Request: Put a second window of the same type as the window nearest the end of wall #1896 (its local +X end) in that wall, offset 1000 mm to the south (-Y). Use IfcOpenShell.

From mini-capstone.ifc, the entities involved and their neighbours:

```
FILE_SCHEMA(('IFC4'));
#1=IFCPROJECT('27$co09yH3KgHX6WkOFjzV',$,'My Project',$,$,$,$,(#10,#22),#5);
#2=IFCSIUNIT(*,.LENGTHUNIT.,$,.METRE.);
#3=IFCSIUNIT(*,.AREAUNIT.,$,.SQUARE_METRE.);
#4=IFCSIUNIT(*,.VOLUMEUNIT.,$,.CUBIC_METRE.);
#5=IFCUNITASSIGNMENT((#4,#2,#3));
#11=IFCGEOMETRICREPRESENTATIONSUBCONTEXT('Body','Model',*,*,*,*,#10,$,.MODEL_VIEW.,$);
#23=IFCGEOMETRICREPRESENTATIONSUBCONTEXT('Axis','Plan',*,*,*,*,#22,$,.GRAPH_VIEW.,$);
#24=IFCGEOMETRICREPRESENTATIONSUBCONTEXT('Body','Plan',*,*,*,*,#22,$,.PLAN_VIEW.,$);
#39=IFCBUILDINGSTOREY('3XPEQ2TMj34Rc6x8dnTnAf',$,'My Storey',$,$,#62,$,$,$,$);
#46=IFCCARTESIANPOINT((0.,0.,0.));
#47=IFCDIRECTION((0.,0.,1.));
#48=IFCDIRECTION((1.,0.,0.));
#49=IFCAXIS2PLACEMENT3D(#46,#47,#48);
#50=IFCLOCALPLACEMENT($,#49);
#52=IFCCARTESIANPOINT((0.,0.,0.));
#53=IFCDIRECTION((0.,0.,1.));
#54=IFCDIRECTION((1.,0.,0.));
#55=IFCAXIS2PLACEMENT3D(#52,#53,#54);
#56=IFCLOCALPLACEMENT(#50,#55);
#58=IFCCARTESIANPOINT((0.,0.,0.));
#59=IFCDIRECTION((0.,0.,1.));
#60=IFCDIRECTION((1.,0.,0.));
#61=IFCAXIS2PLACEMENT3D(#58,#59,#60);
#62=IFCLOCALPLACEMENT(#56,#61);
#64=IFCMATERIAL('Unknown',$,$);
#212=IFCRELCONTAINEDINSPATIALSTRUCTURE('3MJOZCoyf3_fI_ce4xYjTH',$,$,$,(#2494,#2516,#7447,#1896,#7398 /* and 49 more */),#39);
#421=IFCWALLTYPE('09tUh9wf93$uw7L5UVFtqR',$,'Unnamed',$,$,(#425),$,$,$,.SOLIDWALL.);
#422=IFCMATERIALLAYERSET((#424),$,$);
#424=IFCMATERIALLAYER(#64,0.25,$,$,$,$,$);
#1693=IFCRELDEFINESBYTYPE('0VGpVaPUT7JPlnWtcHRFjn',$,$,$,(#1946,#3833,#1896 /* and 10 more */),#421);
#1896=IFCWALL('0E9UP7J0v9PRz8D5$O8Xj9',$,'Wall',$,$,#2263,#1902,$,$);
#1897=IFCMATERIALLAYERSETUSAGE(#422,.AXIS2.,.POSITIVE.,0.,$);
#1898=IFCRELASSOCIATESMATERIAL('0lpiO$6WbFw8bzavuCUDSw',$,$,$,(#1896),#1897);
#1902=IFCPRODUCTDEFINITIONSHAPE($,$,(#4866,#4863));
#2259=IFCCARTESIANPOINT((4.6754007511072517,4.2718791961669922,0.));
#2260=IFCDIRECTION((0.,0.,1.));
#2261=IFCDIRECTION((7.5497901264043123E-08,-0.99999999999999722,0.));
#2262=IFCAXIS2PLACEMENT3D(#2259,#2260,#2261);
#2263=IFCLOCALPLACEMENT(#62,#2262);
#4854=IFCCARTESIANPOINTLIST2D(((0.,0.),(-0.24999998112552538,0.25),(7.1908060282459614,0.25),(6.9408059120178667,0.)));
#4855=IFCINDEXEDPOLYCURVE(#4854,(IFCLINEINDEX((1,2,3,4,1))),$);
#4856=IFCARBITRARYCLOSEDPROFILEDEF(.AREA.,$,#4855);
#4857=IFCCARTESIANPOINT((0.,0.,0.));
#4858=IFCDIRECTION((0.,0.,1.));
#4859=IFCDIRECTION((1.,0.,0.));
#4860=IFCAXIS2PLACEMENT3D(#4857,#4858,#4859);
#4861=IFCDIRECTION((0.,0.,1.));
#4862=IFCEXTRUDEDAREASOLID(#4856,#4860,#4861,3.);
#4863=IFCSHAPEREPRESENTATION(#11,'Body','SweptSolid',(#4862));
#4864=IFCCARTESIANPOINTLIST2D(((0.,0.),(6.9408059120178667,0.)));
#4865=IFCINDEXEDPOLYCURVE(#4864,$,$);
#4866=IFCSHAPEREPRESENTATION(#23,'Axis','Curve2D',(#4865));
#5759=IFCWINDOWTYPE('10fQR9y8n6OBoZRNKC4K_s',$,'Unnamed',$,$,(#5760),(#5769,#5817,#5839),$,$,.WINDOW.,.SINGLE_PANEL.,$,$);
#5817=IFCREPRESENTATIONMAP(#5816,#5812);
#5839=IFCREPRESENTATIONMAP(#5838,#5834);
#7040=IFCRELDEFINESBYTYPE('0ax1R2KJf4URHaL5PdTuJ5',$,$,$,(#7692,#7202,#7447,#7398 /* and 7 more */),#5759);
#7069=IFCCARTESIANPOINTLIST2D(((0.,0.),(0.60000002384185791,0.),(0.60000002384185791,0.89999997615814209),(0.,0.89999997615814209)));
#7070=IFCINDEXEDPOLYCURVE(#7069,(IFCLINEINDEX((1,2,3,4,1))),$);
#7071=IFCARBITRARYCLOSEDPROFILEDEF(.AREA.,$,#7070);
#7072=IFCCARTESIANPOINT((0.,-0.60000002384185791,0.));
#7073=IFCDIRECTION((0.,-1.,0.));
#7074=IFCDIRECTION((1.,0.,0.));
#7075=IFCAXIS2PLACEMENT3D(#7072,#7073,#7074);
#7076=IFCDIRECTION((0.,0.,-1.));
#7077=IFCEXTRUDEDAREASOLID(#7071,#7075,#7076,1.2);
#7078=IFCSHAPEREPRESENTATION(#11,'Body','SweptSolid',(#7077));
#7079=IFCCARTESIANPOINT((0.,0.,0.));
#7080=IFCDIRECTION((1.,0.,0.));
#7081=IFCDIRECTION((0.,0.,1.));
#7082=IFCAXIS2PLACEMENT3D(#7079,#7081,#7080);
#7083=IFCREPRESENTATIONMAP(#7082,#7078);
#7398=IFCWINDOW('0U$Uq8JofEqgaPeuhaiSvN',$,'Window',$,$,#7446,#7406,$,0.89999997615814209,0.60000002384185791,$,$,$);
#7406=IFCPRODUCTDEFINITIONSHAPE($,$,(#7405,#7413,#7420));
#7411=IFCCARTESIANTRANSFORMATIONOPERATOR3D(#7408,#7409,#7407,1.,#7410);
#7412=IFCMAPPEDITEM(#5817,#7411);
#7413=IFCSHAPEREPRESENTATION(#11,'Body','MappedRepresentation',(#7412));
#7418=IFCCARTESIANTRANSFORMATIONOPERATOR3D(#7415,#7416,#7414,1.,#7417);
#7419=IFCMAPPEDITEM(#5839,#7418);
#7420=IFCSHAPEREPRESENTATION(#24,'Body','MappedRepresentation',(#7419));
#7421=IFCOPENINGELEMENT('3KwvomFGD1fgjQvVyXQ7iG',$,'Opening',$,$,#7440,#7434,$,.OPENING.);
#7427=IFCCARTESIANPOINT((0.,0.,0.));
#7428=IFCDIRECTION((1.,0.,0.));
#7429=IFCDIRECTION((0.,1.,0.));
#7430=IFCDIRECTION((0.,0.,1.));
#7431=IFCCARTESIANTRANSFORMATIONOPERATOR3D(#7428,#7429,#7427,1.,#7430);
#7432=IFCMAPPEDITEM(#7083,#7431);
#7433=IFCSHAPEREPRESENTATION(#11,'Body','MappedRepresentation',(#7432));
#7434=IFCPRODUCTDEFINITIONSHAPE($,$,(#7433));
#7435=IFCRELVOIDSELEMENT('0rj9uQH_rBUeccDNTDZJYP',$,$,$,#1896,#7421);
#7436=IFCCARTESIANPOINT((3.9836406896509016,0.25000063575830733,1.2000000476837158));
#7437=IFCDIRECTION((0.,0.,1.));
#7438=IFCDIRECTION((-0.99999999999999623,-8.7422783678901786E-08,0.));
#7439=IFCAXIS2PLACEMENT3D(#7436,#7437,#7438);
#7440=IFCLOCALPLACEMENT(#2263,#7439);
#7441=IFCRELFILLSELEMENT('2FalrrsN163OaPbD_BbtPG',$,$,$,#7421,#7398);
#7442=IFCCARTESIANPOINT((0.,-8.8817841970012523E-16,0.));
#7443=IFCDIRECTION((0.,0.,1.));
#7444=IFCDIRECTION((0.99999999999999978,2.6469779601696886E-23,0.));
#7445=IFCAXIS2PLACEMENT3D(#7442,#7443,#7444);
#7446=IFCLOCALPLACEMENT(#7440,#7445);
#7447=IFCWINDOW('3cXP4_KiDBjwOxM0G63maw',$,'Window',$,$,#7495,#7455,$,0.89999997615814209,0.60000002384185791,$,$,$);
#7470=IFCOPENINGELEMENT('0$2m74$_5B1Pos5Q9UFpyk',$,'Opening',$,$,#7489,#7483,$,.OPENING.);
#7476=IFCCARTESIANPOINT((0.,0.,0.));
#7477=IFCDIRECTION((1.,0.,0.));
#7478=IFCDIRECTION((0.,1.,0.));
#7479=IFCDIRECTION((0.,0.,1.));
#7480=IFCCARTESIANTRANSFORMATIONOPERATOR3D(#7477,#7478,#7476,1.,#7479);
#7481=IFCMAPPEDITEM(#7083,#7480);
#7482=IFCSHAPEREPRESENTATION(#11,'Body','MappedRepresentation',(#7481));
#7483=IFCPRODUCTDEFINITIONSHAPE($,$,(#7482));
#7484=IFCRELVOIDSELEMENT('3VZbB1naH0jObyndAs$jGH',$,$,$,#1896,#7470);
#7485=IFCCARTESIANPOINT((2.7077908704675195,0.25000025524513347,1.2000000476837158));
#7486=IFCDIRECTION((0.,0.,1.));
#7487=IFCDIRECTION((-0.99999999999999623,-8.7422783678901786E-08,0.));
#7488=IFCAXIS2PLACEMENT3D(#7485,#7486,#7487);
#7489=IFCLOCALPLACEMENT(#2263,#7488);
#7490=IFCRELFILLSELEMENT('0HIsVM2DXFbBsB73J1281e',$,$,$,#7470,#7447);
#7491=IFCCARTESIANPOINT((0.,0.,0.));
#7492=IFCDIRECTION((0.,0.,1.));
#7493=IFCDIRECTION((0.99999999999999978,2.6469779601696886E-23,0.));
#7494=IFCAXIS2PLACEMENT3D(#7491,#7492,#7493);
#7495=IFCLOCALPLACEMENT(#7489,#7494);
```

```python
import ifcopenshell
import ifcopenshell.api.feature
import ifcopenshell.api.geometry
import ifcopenshell.api.root
import ifcopenshell.geom
import ifcopenshell.util.element
import ifcopenshell.util.placement
import ifcopenshell.util.shape
import ifcopenshell.util.unit

model = ifcopenshell.open("mini-capstone.ifc")
unit_scale = ifcopenshell.util.unit.calculate_unit_scale(model)
settings = ifcopenshell.geom.settings()


def volume(element):
    """Net volume in cubic metres, openings subtracted."""
    shape = ifcopenshell.geom.create_shape(settings, element)
    return ifcopenshell.util.shape.get_volume(shape.geometry)


window = model.by_guid("0U$Uq8JofEqgaPeuhaiSvN")
opening = window.FillsVoids[0].RelatingOpeningElement
wall = opening.VoidsElements[0].RelatingBuildingElement
before = volume(wall)
shift = ifcopenshell.util.placement.get_local_placement(wall.ObjectPlacement)[:3, 0] * 1 / unit_scale

# copy_class copies the void relationship, type, container and properties, but no geometry.
new_opening = ifcopenshell.api.root.copy_class(model, product=opening)
new_opening.Representation = ifcopenshell.util.element.copy_deep(
    model, opening.Representation, exclude=["IfcGeometricRepresentationContext", "IfcRepresentationMap"]
)
new_window = ifcopenshell.api.root.copy_class(model, product=window)
new_window.Representation = ifcopenshell.util.element.copy_deep(
    model, window.Representation, exclude=["IfcGeometricRepresentationContext", "IfcRepresentationMap"]
)
ifcopenshell.api.feature.add_filling(model, opening=new_opening, element=new_window)

for old, new in ((opening, new_opening), (window, new_window)):
    matrix = ifcopenshell.util.placement.get_local_placement(old.ObjectPlacement)
    matrix[:3, 3] += shift
    ifcopenshell.api.geometry.edit_object_placement(model, product=new, matrix=matrix, is_si=False)

after = volume(wall)

print(f"wall volume {before:.3f} -> {after:.3f} m3")

model.write("mini-capstone_edited.ifc")
```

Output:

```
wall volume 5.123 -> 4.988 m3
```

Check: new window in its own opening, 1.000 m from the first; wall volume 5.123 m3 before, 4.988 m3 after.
